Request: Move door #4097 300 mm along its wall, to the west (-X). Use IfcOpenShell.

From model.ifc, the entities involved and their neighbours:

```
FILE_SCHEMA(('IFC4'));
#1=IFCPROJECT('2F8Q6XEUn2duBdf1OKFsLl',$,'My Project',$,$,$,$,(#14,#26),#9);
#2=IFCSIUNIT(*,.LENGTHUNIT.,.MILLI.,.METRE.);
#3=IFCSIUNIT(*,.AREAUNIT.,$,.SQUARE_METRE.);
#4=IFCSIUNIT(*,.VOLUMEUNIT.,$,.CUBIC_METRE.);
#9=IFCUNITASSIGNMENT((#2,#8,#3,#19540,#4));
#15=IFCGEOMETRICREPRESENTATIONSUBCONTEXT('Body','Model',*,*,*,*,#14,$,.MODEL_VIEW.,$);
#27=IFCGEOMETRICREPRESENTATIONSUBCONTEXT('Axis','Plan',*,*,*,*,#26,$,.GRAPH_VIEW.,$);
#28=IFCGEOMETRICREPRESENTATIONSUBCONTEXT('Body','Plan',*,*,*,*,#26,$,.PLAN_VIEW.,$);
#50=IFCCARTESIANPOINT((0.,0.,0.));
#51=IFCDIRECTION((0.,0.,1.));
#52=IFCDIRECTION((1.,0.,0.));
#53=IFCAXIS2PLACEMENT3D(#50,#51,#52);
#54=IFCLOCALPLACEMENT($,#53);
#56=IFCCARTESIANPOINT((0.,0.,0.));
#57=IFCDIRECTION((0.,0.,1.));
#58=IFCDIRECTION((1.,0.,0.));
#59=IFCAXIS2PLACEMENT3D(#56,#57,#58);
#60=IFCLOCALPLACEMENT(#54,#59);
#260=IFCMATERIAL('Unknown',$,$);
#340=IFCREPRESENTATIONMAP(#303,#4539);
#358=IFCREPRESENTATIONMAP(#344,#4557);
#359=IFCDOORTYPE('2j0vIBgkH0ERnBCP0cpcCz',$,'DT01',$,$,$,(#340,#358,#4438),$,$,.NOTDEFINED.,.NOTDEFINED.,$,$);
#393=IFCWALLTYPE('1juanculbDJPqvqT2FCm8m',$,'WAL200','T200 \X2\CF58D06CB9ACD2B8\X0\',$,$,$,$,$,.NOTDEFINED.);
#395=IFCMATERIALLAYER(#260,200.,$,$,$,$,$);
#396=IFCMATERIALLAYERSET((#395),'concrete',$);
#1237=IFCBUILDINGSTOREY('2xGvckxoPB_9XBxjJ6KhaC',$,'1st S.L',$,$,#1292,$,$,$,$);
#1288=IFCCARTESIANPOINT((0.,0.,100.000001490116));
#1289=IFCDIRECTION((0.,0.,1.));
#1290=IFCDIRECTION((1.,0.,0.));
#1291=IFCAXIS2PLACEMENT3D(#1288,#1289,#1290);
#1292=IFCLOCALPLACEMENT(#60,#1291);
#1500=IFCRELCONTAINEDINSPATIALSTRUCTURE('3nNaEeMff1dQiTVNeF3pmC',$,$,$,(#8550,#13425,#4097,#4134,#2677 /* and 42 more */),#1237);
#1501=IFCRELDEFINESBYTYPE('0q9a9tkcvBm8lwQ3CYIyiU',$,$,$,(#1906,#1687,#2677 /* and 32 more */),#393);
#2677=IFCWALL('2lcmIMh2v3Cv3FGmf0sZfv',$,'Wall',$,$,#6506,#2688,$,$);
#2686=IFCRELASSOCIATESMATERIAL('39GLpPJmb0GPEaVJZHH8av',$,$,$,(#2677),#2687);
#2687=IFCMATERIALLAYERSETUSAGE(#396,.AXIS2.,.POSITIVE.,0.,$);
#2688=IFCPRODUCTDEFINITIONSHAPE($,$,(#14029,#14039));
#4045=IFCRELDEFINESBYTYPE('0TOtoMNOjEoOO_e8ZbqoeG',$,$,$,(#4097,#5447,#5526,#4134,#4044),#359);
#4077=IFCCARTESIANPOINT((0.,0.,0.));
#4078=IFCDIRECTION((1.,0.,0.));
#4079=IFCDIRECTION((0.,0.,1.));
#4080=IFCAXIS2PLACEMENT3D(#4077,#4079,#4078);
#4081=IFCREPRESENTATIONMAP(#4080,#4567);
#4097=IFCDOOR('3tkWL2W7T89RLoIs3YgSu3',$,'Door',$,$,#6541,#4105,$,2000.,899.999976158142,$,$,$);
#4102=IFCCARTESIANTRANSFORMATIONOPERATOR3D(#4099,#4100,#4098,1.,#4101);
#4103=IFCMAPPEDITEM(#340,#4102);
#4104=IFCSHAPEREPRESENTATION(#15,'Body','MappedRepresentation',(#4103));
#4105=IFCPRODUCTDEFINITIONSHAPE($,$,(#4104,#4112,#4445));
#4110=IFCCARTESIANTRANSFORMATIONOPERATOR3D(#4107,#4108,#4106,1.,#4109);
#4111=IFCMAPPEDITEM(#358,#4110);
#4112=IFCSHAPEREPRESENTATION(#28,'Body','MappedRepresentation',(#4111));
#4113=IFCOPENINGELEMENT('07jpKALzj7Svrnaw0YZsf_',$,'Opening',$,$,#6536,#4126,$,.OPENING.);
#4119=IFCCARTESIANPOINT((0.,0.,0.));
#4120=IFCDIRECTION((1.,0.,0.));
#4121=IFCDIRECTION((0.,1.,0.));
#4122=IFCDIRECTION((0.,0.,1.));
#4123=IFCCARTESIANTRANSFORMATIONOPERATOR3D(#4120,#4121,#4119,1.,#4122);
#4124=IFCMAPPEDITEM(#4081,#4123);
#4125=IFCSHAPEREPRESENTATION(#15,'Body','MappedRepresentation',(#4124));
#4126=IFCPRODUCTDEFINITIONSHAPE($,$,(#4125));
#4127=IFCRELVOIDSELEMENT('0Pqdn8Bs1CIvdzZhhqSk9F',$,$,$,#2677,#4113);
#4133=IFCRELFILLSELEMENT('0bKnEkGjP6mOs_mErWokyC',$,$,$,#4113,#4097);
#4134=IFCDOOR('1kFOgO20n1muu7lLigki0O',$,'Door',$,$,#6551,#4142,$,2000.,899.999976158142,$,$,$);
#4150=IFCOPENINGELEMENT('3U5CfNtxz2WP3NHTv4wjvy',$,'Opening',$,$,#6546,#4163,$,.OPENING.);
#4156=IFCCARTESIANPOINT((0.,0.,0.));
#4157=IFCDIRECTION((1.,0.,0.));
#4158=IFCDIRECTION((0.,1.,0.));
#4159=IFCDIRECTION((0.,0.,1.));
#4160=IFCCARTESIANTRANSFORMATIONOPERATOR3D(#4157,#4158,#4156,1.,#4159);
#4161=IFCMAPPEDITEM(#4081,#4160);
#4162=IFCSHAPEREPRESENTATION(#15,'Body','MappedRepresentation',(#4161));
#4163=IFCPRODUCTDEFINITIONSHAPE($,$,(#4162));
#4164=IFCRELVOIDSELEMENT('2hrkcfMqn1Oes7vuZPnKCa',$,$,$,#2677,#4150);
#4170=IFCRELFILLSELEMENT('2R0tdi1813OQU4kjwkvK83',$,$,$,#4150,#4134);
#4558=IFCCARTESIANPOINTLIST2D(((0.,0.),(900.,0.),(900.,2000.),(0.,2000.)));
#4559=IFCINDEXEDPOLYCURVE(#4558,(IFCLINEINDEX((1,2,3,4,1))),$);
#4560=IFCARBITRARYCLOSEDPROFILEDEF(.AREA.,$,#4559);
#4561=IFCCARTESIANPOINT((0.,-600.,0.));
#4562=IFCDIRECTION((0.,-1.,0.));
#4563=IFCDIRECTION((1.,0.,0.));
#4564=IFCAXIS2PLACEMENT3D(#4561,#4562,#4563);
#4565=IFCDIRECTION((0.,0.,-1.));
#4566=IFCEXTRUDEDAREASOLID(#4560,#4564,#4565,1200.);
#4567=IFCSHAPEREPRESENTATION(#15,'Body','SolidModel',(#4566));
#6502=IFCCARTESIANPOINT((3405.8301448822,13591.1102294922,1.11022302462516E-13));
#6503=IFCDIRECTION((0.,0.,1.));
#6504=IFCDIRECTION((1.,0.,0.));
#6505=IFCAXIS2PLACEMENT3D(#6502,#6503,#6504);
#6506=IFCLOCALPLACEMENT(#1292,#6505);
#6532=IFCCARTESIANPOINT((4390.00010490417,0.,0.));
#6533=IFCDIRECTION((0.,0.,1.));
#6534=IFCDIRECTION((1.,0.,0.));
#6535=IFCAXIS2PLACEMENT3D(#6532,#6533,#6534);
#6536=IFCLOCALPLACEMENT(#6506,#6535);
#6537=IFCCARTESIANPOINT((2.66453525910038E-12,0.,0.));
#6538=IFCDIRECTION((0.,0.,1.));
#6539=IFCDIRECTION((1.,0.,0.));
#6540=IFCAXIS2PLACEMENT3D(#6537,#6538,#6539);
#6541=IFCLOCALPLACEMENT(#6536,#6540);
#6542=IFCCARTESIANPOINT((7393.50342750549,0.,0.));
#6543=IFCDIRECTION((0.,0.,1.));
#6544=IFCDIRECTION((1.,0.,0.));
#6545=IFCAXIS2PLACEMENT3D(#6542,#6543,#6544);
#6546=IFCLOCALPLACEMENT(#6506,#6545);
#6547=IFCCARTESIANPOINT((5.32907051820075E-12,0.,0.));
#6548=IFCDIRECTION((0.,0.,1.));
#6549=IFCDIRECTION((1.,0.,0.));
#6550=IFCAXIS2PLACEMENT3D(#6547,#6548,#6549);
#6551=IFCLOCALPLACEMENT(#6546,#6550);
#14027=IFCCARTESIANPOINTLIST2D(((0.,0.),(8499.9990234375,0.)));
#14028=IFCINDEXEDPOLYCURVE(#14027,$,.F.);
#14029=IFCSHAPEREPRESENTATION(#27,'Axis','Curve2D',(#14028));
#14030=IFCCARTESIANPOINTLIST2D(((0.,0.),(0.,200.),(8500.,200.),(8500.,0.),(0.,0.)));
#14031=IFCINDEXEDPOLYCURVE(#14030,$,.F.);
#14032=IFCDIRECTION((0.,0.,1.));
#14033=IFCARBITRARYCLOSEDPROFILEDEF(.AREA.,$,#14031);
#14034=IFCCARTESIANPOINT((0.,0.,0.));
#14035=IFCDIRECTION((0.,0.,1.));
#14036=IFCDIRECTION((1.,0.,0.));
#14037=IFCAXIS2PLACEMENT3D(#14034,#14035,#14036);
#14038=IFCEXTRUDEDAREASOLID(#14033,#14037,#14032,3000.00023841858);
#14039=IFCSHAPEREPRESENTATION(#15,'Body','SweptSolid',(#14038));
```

```python
import ifcopenshell
import ifcopenshell.api.geometry
import ifcopenshell.util.placement
import ifcopenshell.util.unit

model = ifcopenshell.open("model.ifc")
unit_scale = ifcopenshell.util.unit.calculate_unit_scale(model)

door = model.by_id(4097)
opening = door.FillsVoids[0].RelatingOpeningElement
wall = opening.VoidsElements[0].RelatingBuildingElement

wall_matrix = ifcopenshell.util.placement.get_local_placement(wall.ObjectPlacement)
shift = wall_matrix[:3, 0] * -0.3 / unit_scale
before = ifcopenshell.util.placement.get_local_placement(door.ObjectPlacement)[:3, 3].copy()

# The door is placed relative to its opening, so it follows when the opening moves.
matrix = ifcopenshell.util.placement.get_local_placement(opening.ObjectPlacement)
matrix[:3, 3] += shift
ifcopenshell.api.geometry.edit_object_placement(
    model, product=opening, matrix=matrix, is_si=False, should_transform_children=True
)

after = ifcopenshell.util.placement.get_local_placement(door.ObjectPlacement)[:3, 3]
print("door moved by", (after - before).round(3) + 0.0)

model.write("model_v2.ifc")
```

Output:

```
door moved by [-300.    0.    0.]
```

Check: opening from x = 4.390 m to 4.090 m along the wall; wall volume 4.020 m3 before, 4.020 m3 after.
